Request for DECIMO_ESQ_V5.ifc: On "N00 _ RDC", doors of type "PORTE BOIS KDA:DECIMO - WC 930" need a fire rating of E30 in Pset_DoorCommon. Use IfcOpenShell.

First a look at what the model holds.

```python
import ifcopenshell
import ifcopenshell.util.element

model = ifcopenshell.open("DECIMO_ESQ_V5.ifc")
print(model.schema)
storey = next(s for s in model.by_type("IfcBuildingStorey") if s.Name == "N00 _ RDC")
doors = [e for e in ifcopenshell.util.element.get_decomposition(storey) if e.is_a("IfcDoor")]
seen = {}
for e in doors:
    element_type = ifcopenshell.util.element.get_type(e)
    key = (element_type.Name if element_type != e and element_type else None, ifcopenshell.util.element.get_pset(e, "Pset_DoorCommon", "FireRating"))
    seen[key] = seen.get(key, 0) + 1
for (name, value), count in sorted(seen.items(), key=str):
    print(count, "x", name, "|", value)
```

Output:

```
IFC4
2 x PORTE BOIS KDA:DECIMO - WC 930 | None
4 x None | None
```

```python
import ifcopenshell
import ifcopenshell.api.pset
import ifcopenshell.util.element

model = ifcopenshell.open("DECIMO_ESQ_V5.ifc")

storey = next(s for s in model.by_type("IfcBuildingStorey") if s.Name == "N00 _ RDC")
doors = [e for e in ifcopenshell.util.element.get_decomposition(storey) if e.is_a("IfcDoor")]

count = 0
for e in doors:
    element_type = ifcopenshell.util.element.get_type(e)
    if element_type in (None, e) or element_type.Name != "PORTE BOIS KDA:DECIMO - WC 930":
        continue
    # add_pset returns the element's existing set when there is one.
    pset = ifcopenshell.api.pset.add_pset(model, product=e, name="Pset_DoorCommon")
    ifcopenshell.api.pset.edit_pset(model, pset=pset, properties={"FireRating": "E30"})
    count += 1

print(count, "doors updated")

model.write("DECIMO_ESQ_V5_v2.ifc")
```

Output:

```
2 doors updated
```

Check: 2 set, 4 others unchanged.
